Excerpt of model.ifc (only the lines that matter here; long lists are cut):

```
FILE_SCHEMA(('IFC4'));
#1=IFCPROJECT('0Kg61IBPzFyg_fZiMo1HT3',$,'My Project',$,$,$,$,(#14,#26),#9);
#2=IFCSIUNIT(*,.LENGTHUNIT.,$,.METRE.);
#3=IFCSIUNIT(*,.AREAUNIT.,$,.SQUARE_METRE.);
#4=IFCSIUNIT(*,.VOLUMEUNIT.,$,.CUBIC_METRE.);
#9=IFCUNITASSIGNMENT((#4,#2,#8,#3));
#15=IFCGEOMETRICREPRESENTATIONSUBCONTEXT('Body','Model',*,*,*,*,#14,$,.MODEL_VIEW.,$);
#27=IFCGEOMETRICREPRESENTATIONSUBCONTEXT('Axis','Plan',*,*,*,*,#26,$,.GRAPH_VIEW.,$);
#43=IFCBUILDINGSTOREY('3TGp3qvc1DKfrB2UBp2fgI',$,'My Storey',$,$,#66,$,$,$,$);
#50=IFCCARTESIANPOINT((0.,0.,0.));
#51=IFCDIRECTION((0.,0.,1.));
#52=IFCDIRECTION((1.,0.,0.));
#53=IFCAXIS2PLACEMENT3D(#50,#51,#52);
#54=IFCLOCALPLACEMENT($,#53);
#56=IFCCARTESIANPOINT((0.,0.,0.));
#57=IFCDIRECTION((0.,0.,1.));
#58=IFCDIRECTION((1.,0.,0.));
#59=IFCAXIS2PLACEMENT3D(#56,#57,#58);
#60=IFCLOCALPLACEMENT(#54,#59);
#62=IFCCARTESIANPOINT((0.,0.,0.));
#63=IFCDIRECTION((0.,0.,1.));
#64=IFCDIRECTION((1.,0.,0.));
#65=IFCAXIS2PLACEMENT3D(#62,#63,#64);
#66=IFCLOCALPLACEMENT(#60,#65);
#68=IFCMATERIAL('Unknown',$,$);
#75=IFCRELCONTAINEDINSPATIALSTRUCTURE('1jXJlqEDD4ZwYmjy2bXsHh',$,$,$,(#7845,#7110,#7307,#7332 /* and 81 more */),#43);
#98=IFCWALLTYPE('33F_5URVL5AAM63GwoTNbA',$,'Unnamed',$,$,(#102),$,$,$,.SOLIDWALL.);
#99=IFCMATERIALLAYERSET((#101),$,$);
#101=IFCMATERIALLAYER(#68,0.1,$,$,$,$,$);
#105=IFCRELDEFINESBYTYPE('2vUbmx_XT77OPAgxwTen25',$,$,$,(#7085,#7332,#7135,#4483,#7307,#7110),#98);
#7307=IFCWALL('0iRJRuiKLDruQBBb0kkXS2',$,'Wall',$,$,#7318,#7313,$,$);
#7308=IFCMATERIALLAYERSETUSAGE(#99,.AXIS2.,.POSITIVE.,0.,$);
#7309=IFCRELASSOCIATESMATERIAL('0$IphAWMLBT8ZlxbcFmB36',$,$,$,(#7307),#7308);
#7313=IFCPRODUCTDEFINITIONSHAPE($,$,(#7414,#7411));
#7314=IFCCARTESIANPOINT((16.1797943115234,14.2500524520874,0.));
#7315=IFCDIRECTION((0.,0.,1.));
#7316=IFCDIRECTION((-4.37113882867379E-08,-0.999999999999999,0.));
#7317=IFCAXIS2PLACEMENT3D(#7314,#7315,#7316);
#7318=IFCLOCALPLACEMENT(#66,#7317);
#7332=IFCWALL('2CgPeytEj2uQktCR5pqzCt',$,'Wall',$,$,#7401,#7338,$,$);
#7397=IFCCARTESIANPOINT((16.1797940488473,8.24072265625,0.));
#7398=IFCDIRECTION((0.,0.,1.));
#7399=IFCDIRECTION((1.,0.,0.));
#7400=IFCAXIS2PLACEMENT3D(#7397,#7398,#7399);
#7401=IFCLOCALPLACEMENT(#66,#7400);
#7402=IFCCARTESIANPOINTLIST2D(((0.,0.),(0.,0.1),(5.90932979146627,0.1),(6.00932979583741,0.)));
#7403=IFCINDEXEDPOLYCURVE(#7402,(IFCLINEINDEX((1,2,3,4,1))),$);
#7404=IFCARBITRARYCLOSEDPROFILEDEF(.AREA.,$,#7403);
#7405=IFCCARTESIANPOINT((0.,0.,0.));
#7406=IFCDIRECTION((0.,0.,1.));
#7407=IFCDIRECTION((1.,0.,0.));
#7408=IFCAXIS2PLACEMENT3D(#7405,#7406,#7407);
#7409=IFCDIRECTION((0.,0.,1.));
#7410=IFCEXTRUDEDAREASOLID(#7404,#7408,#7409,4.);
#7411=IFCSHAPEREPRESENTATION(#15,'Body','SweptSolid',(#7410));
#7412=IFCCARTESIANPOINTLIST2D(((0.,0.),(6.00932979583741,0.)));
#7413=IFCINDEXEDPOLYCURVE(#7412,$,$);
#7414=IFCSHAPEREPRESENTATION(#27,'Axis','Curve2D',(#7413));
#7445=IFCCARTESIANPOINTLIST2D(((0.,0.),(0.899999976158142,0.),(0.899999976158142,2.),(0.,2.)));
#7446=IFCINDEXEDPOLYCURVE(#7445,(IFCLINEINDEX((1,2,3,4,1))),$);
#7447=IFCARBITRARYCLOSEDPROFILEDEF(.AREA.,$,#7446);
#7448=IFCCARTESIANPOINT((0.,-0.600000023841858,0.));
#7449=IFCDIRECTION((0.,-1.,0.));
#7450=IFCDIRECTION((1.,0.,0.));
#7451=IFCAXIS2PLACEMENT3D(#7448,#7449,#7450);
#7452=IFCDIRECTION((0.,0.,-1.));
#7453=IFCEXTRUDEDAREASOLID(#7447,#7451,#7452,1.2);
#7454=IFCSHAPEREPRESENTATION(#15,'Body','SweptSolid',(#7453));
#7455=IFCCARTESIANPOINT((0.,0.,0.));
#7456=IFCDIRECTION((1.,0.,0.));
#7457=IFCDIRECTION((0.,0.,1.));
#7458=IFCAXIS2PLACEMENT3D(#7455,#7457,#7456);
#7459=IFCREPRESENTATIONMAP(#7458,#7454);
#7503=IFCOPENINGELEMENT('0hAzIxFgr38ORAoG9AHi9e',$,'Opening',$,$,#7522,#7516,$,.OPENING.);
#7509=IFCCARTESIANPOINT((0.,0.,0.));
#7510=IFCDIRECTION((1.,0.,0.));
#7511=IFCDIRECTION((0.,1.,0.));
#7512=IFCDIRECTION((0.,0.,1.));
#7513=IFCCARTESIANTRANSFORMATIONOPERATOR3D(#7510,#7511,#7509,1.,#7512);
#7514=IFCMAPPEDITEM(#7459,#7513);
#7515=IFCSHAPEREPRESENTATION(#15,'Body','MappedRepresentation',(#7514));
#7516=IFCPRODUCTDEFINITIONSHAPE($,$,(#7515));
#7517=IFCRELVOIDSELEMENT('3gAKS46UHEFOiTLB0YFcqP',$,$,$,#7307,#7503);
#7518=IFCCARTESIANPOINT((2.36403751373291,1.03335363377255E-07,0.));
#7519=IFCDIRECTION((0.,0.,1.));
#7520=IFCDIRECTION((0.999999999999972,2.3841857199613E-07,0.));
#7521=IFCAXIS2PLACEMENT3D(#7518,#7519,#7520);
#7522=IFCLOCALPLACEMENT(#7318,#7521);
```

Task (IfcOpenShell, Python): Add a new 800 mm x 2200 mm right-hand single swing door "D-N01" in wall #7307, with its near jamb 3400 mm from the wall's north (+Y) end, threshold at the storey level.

```python
import numpy as np
import ifcopenshell
import ifcopenshell.api.feature
import ifcopenshell.api.geometry
import ifcopenshell.api.root
import ifcopenshell.api.spatial
import ifcopenshell.geom
import ifcopenshell.util.element
import ifcopenshell.util.placement
import ifcopenshell.util.representation
import ifcopenshell.util.shape
import ifcopenshell.util.unit

model = ifcopenshell.open("model.ifc")
unit_scale = ifcopenshell.util.unit.calculate_unit_scale(model)
settings = ifcopenshell.geom.settings()


def volume(element):
    """Net volume in cubic metres, openings subtracted."""
    shape = ifcopenshell.geom.create_shape(settings, element)
    return ifcopenshell.util.shape.get_volume(shape.geometry)


wall = model.by_guid("0iRJRuiKLDruQBBb0kkXS2")
storey = ifcopenshell.util.element.get_container(wall, ifc_class="IfcBuildingStorey")
context = ifcopenshell.util.representation.get_context(model, "Model", "Body", "MODEL_VIEW")
before = volume(wall)

width, height, from_end, sill = 0.8, 2.2, 3.4, 0.0  # metres

# The wall runs along its own X axis, and the end named is its -X end.
wall_shape = ifcopenshell.geom.create_shape(settings, wall)
x, y, z = ifcopenshell.util.shape.get_vertices(wall_shape.geometry).T
start = x.min() + from_end
face, thickness = float(y.min()), float(y.max() - y.min())
wall_matrix = ifcopenshell.util.placement.get_local_placement(wall.ObjectPlacement)
level = ifcopenshell.util.placement.get_local_placement(storey.ObjectPlacement)[2, 3]


def in_wall(x, y):
    """Placement at x, y metres in the wall's axes, at sill height."""
    matrix = wall_matrix.copy()
    matrix[:, 3] = wall_matrix @ np.array([x / unit_scale, y / unit_scale, 0.0, 1.0])
    matrix[2, 3] = level + sill / unit_scale
    return matrix


# Opening: a box that overshoots both wall faces by 50 mm.
opening = ifcopenshell.api.root.create_entity(model, ifc_class="IfcOpeningElement", predefined_type="OPENING")
box = ifcopenshell.api.geometry.add_wall_representation(
    model, context=context, length=width, height=height, thickness=thickness + 0.1
)
ifcopenshell.api.geometry.assign_representation(model, product=opening, representation=box)
ifcopenshell.api.geometry.edit_object_placement(model, product=opening, matrix=in_wall(start, face - 0.05), is_si=False)
ifcopenshell.api.feature.add_feature(model, feature=opening, element=wall)

door = ifcopenshell.api.root.create_entity(model, ifc_class="IfcDoor", name="D-N01", predefined_type="DOOR")
door.OverallWidth, door.OverallHeight = width / unit_scale, height / unit_scale
door.OperationType = "SINGLE_SWING_RIGHT"
body = ifcopenshell.api.geometry.add_door_representation(
    model,
    context=context,
    overall_width=door.OverallWidth,
    overall_height=door.OverallHeight,
    operation_type="SINGLE_SWING_RIGHT",
    lining_properties={"LiningDepth": thickness / unit_scale, "ThresholdDepth": thickness / unit_scale},
)
ifcopenshell.api.geometry.assign_representation(model, product=door, representation=body)
ifcopenshell.api.spatial.assign_container(model, products=[door], relating_structure=storey)
ifcopenshell.api.feature.add_filling(model, opening=opening, element=door)

# The lining spans the wall, so the door starts at the wall face.
ifcopenshell.api.geometry.edit_object_placement(model, product=door, matrix=in_wall(start, face), is_si=False)

after = volume(wall)

print(f"wall volume {before:.3f} -> {after:.3f} m3")

model.write("model_edited.ifc")
```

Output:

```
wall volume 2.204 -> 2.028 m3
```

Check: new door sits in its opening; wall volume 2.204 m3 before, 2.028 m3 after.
